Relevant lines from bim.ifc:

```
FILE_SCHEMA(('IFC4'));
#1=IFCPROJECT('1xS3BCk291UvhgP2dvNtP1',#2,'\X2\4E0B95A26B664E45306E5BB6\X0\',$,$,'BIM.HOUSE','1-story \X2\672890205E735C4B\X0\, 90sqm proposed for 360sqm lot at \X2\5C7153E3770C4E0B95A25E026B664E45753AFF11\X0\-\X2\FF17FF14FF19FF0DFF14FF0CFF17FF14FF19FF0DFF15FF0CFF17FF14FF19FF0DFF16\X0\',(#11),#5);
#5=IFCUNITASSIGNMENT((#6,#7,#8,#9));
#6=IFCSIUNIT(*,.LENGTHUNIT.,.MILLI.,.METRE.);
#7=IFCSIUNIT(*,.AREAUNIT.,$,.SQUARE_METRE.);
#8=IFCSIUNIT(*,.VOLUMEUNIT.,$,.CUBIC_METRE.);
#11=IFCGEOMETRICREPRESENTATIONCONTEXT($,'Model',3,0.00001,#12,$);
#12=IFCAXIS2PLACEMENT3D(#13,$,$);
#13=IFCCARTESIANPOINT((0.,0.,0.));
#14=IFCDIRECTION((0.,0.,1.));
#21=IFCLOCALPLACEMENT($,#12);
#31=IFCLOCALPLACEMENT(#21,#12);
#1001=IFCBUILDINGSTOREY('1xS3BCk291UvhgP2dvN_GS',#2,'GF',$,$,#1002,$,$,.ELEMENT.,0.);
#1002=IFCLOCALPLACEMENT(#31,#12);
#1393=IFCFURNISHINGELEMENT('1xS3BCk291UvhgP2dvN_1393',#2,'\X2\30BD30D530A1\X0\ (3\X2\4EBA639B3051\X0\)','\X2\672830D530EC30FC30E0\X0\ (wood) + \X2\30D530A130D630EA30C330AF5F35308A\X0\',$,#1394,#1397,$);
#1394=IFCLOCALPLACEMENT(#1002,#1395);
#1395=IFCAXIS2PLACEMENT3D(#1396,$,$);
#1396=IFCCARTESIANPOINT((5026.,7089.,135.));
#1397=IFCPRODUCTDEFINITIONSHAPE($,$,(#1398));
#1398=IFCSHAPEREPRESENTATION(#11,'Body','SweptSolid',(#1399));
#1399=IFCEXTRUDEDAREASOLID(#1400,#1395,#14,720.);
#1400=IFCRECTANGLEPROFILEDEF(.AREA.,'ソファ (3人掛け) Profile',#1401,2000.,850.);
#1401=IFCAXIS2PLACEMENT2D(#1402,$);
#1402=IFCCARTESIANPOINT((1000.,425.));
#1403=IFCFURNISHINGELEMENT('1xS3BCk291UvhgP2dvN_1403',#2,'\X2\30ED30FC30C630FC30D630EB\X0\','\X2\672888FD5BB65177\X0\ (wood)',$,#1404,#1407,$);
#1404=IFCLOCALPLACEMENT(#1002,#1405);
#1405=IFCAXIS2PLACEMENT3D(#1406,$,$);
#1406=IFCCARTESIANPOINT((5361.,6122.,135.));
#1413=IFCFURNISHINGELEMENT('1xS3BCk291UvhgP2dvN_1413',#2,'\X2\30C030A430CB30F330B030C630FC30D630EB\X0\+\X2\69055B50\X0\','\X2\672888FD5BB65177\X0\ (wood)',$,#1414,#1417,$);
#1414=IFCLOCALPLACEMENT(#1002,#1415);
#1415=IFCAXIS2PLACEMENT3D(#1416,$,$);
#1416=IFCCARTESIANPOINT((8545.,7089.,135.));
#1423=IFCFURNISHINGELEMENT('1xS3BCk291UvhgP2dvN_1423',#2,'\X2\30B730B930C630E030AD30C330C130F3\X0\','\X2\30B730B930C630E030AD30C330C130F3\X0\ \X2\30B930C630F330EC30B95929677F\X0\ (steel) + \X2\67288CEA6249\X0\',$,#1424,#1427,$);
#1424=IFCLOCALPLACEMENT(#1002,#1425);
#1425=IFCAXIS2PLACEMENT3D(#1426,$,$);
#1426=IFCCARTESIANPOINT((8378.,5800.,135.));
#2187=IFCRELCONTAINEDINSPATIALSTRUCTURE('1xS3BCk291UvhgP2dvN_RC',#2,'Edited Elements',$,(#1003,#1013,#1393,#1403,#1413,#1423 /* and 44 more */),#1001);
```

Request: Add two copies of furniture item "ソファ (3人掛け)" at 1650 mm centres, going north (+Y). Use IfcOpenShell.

```python
import numpy as np
import ifcopenshell
import ifcopenshell.api.geometry
import ifcopenshell.api.root
import ifcopenshell.util.element
import ifcopenshell.util.placement

model = ifcopenshell.open("bim.ifc")


def reuse_history(source, copy):
    """copy_class also copies each property set's owner history, people and application; keep the originals."""
    for rel in copy.IsDefinedBy:
        if rel.is_a("IfcRelDefinesByProperties") and (history := rel.RelatingPropertyDefinition.OwnerHistory):
            rel.RelatingPropertyDefinition.OwnerHistory = source.OwnerHistory
            ifcopenshell.util.element.remove_deep2(model, history)


source = model.by_guid("1xS3BCk291UvhgP2dvN_1393")
base = ifcopenshell.util.placement.get_local_placement(source.ObjectPlacement)
step = np.array([0.0, 1.0, 0.0]) * 1650.0

for i in range(1, 3):
    copy = ifcopenshell.api.root.copy_class(model, product=source)
    copy.Representation = ifcopenshell.util.element.copy_deep(
        model, source.Representation, exclude=["IfcGeometricRepresentationContext", "IfcRepresentationMap"]
    )
    reuse_history(source, copy)
    matrix = base.copy()
    matrix[:3, 3] += i * step
    print("added at", matrix[:3, 3].round(3) + 0.0)
    ifcopenshell.api.geometry.edit_object_placement(model, product=copy, matrix=matrix, is_si=False)

model.write("bim_edited.ifc")
```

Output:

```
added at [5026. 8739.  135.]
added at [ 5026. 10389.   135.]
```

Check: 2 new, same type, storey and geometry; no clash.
